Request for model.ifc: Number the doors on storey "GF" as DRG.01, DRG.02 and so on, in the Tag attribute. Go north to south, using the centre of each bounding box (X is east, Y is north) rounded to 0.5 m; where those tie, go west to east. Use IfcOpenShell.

First a look at what the model holds.

```python
import ifcopenshell
import ifcopenshell.util.element
import ifcopenshell.util.placement

model = ifcopenshell.open("model.ifc")
print(model.schema)
storey = next(s for s in model.by_type("IfcBuildingStorey") if s.Name == "GF")
doors = [e for e in ifcopenshell.util.element.get_decomposition(storey) if e.is_a("IfcDoor")]
for e in sorted(doors, key=lambda e: e.id()):
    origin = ifcopenshell.util.placement.get_local_placement(e.ObjectPlacement)[:3, 3]
    print(e.id(), e.Tag, e.Name, origin.round(2) + 0.0, sep=" | ")
```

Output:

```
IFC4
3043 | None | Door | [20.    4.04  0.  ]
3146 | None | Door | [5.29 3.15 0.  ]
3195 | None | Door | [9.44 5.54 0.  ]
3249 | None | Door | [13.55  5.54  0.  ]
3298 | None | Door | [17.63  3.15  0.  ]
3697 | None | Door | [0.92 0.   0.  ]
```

```python
import ifcopenshell
import ifcopenshell.geom
import ifcopenshell.util.element
import ifcopenshell.util.shape

model = ifcopenshell.open("model.ifc")
settings = ifcopenshell.geom.settings()
settings.set("use-world-coords", True)


def centre(element):
    shape = ifcopenshell.geom.create_shape(settings, element)
    return ifcopenshell.util.shape.get_bbox_centroid(shape.geometry)


storey = next(s for s in model.by_type("IfcBuildingStorey") if s.Name == "GF")
doors = [e for e in ifcopenshell.util.element.get_decomposition(storey) if e.is_a("IfcDoor")]

# Insertion points can sit at a corner or the storey origin, so sort by the geometry (in metres).
centres = {e: centre(e) for e in doors}
doors.sort(key=lambda e: (-round(centres[e][1] / 0.5), centres[e][0]))

for i, e in enumerate(doors, start=1):
    number = f"DRG.{i:02d}"
    e.Tag = number
    print(e.id(), number)

model.write("model_edited.ifc")
```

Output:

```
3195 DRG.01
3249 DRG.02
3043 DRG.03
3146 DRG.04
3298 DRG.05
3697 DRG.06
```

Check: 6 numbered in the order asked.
